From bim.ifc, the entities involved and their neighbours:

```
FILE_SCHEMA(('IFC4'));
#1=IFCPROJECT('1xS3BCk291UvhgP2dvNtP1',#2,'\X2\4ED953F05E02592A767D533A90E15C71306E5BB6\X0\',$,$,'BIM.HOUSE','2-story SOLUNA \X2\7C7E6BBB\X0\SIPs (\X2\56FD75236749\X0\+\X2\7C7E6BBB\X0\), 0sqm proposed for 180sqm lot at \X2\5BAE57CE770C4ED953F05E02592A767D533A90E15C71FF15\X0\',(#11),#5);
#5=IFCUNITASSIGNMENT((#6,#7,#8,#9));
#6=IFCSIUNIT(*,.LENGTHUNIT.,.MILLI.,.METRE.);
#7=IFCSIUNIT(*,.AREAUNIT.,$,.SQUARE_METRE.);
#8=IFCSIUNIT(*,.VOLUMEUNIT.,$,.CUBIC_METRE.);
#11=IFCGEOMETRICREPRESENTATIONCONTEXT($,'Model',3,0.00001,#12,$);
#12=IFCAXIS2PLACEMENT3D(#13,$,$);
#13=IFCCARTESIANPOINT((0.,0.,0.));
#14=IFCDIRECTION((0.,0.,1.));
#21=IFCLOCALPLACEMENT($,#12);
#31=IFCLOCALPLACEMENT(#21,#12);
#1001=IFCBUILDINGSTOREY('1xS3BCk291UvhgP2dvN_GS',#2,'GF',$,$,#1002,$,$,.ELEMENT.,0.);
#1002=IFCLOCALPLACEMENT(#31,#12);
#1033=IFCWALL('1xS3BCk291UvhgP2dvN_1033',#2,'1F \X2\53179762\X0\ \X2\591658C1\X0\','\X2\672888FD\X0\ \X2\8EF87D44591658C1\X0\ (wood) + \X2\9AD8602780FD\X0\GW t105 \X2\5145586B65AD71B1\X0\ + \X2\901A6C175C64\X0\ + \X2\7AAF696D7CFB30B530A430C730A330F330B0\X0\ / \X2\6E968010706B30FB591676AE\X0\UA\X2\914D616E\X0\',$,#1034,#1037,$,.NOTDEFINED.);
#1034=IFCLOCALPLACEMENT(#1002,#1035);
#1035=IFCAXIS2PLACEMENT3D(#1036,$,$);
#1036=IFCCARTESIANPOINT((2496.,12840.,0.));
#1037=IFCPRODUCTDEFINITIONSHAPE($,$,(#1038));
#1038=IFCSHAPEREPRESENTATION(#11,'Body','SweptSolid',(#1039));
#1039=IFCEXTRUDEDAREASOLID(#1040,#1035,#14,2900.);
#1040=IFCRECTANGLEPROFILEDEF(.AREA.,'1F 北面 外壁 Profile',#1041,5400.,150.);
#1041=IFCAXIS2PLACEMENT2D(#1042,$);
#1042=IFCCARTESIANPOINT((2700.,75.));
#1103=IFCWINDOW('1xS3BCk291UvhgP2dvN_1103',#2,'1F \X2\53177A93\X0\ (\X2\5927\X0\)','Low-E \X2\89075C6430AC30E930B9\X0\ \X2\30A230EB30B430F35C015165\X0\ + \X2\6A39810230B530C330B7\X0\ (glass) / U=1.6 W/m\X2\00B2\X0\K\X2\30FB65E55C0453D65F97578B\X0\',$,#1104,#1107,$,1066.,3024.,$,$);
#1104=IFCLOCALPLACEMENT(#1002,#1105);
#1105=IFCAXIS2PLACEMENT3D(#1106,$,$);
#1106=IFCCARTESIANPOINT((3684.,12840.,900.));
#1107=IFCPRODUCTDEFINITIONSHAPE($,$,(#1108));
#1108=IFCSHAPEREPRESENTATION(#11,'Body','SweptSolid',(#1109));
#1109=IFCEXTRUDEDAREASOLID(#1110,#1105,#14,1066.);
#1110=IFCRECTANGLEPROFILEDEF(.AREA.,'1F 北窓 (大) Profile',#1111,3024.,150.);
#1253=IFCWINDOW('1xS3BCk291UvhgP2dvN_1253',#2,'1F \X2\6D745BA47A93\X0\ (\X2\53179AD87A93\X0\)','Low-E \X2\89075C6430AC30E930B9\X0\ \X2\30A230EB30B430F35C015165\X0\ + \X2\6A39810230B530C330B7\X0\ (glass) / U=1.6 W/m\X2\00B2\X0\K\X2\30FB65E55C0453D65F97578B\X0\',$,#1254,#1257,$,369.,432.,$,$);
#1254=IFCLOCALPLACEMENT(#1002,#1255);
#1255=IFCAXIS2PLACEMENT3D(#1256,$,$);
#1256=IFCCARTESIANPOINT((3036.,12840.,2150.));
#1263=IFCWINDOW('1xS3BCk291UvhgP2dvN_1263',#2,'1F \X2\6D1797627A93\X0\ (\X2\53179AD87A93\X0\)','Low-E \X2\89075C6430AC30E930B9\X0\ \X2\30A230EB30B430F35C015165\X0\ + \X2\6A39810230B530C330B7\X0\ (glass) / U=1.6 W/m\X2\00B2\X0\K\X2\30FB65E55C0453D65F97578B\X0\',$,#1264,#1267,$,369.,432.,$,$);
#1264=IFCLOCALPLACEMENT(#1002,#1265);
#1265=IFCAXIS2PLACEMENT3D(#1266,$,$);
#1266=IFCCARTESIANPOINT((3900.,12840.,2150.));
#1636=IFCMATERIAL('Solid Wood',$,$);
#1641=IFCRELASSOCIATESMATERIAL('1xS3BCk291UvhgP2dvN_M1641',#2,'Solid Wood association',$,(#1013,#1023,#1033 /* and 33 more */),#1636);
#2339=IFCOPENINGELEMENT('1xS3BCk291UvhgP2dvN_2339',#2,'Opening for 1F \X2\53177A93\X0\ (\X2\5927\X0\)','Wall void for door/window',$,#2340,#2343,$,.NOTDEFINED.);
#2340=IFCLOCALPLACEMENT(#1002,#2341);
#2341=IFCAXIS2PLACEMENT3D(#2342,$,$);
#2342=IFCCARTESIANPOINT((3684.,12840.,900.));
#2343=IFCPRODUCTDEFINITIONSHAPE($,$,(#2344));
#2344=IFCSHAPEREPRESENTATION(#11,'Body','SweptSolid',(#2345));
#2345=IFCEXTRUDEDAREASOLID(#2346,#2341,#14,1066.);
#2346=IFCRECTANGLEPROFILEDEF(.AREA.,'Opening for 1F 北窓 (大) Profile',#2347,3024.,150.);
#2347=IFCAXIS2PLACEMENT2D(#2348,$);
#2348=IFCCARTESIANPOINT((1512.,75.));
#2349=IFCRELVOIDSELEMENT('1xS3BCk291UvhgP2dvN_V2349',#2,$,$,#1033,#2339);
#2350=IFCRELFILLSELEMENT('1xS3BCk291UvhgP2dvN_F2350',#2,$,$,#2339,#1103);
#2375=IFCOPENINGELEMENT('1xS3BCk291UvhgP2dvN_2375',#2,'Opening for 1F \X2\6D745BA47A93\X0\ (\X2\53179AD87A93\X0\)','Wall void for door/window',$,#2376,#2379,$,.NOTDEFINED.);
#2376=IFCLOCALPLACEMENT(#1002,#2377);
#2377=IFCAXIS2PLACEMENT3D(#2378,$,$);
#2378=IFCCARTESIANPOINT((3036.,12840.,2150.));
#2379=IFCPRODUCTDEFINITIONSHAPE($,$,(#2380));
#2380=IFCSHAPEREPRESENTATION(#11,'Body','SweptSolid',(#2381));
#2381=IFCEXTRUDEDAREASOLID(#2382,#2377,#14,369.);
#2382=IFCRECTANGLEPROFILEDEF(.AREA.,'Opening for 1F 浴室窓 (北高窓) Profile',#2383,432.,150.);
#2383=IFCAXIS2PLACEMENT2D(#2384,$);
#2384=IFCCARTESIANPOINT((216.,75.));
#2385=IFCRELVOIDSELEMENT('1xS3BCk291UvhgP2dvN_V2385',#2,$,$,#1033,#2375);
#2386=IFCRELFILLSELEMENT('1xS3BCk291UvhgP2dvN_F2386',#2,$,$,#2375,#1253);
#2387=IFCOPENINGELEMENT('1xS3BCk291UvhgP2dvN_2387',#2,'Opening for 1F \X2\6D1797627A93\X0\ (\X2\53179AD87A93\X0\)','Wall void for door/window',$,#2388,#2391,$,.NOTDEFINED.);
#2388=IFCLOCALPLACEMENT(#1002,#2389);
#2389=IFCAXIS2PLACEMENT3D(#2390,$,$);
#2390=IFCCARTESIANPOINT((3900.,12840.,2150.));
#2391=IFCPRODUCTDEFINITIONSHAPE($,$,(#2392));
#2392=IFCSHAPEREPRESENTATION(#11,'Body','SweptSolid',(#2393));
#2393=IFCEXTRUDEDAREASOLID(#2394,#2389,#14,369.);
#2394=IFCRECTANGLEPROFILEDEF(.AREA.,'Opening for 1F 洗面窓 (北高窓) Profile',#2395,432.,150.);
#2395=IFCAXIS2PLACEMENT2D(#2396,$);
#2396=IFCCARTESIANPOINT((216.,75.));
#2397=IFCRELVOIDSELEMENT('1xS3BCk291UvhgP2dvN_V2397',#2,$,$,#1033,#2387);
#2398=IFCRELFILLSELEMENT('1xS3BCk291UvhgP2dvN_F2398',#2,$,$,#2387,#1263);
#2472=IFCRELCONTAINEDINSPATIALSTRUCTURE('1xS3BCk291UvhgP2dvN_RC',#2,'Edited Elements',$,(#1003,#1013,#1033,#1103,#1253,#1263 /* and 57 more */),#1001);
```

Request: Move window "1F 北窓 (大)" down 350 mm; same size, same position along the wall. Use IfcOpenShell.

```python
import numpy as np
import ifcopenshell
import ifcopenshell.api.geometry
import ifcopenshell.util.placement
import ifcopenshell.util.unit

model = ifcopenshell.open("bim.ifc")
unit_scale = ifcopenshell.util.unit.calculate_unit_scale(model)

window = model.by_guid("1xS3BCk291UvhgP2dvN_1103")
opening = window.FillsVoids[0].RelatingOpeningElement
dz = -350.0

shift = np.array([0.0, 0.0, dz])
# The window is not placed relative to its opening, so move both.
for product in (opening, window):
    matrix = ifcopenshell.util.placement.get_local_placement(product.ObjectPlacement)
    matrix[:3, 3] += shift
    ifcopenshell.api.geometry.edit_object_placement(model, product=product, matrix=matrix, is_si=False)

print(f"moved by {dz * unit_scale:+.3f} m")

model.write("bim_v2.ifc")
```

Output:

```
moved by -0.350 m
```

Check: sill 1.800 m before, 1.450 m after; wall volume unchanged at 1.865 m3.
